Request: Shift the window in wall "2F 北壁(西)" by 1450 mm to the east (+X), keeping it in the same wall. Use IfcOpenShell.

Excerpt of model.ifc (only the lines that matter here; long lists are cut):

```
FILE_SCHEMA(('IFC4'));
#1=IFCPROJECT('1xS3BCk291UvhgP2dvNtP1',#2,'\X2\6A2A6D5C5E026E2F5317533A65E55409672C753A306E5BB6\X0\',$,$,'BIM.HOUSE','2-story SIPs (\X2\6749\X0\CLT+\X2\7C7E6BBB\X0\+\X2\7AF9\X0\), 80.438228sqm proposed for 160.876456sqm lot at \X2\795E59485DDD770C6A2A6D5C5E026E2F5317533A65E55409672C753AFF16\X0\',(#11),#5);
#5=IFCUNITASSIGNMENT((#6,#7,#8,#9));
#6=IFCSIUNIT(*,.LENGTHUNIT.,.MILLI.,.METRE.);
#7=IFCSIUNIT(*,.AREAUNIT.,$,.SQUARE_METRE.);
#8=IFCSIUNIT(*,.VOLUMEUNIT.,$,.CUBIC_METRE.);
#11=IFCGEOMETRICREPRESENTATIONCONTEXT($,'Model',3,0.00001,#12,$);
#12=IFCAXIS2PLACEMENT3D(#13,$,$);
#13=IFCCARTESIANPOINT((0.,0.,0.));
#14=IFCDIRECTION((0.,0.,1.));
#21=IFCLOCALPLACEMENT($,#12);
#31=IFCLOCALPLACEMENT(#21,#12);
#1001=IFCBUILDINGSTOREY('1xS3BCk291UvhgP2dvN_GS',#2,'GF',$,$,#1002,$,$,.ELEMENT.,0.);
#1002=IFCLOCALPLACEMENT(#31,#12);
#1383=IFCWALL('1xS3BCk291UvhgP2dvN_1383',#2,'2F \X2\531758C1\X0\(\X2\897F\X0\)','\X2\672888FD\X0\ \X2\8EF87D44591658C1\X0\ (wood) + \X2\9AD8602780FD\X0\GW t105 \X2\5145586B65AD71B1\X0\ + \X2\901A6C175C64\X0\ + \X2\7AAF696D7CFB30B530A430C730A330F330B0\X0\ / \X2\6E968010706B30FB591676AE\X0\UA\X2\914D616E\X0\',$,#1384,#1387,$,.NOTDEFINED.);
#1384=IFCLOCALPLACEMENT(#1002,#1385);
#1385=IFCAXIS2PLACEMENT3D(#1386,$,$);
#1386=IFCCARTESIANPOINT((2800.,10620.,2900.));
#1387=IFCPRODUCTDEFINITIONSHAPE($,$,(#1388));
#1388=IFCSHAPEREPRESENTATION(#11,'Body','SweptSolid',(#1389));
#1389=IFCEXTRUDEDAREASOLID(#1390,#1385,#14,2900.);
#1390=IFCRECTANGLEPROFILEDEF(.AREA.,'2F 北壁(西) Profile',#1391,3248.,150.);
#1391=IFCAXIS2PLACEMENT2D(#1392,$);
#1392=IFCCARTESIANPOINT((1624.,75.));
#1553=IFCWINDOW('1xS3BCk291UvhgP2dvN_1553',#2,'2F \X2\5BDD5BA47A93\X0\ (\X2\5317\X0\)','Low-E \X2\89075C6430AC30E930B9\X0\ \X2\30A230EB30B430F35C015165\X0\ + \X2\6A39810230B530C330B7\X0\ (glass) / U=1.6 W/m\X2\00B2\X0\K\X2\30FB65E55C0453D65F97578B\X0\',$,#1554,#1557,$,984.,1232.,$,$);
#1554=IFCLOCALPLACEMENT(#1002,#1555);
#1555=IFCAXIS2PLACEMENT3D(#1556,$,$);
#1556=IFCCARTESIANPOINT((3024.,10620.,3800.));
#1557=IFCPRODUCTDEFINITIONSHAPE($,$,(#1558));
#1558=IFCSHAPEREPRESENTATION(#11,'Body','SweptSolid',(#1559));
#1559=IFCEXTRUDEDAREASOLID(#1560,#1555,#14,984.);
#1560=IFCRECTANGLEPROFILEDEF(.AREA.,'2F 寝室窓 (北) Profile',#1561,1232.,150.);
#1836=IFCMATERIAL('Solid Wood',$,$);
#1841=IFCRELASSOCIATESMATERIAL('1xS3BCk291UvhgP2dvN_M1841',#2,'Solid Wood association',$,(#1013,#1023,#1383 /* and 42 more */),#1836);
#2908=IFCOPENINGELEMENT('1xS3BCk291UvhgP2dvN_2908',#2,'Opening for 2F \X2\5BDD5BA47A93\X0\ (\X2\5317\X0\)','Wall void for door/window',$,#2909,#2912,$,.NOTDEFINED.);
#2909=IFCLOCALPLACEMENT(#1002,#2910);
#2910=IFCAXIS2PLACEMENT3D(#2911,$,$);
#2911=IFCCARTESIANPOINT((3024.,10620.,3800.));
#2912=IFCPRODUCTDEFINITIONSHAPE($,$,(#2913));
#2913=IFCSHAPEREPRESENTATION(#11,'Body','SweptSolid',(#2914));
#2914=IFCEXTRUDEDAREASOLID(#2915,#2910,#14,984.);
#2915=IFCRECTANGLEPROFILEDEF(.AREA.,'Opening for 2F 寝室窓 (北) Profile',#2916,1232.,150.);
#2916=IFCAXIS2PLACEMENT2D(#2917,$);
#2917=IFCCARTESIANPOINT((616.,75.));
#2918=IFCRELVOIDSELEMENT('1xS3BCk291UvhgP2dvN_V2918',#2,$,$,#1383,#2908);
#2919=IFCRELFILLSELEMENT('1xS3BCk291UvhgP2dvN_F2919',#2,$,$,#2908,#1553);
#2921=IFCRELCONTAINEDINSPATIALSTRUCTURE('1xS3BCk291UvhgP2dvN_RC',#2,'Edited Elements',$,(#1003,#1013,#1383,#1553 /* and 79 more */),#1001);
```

```python
import ifcopenshell
import ifcopenshell.api.geometry
import ifcopenshell.util.placement
import ifcopenshell.util.unit

model = ifcopenshell.open("model.ifc")
unit_scale = ifcopenshell.util.unit.calculate_unit_scale(model)

window = model.by_guid("1xS3BCk291UvhgP2dvN_1553")
opening = window.FillsVoids[0].RelatingOpeningElement
wall = opening.VoidsElements[0].RelatingBuildingElement

wall_matrix = ifcopenshell.util.placement.get_local_placement(wall.ObjectPlacement)
shift = wall_matrix[:3, 0] * 1.45 / unit_scale
before = ifcopenshell.util.placement.get_local_placement(window.ObjectPlacement)[:3, 3].copy()

# The window is not placed relative to its opening, so move both.
for product in (opening, window):
    matrix = ifcopenshell.util.placement.get_local_placement(product.ObjectPlacement)
    matrix[:3, 3] += shift
    ifcopenshell.api.geometry.edit_object_placement(model, product=product, matrix=matrix, is_si=False)

after = ifcopenshell.util.placement.get_local_placement(window.ObjectPlacement)[:3, 3]
print("window moved by", (after - before).round(3) + 0.0)

model.write("model_edited.ifc")
```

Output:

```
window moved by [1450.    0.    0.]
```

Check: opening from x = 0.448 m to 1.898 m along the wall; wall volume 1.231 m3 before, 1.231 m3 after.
